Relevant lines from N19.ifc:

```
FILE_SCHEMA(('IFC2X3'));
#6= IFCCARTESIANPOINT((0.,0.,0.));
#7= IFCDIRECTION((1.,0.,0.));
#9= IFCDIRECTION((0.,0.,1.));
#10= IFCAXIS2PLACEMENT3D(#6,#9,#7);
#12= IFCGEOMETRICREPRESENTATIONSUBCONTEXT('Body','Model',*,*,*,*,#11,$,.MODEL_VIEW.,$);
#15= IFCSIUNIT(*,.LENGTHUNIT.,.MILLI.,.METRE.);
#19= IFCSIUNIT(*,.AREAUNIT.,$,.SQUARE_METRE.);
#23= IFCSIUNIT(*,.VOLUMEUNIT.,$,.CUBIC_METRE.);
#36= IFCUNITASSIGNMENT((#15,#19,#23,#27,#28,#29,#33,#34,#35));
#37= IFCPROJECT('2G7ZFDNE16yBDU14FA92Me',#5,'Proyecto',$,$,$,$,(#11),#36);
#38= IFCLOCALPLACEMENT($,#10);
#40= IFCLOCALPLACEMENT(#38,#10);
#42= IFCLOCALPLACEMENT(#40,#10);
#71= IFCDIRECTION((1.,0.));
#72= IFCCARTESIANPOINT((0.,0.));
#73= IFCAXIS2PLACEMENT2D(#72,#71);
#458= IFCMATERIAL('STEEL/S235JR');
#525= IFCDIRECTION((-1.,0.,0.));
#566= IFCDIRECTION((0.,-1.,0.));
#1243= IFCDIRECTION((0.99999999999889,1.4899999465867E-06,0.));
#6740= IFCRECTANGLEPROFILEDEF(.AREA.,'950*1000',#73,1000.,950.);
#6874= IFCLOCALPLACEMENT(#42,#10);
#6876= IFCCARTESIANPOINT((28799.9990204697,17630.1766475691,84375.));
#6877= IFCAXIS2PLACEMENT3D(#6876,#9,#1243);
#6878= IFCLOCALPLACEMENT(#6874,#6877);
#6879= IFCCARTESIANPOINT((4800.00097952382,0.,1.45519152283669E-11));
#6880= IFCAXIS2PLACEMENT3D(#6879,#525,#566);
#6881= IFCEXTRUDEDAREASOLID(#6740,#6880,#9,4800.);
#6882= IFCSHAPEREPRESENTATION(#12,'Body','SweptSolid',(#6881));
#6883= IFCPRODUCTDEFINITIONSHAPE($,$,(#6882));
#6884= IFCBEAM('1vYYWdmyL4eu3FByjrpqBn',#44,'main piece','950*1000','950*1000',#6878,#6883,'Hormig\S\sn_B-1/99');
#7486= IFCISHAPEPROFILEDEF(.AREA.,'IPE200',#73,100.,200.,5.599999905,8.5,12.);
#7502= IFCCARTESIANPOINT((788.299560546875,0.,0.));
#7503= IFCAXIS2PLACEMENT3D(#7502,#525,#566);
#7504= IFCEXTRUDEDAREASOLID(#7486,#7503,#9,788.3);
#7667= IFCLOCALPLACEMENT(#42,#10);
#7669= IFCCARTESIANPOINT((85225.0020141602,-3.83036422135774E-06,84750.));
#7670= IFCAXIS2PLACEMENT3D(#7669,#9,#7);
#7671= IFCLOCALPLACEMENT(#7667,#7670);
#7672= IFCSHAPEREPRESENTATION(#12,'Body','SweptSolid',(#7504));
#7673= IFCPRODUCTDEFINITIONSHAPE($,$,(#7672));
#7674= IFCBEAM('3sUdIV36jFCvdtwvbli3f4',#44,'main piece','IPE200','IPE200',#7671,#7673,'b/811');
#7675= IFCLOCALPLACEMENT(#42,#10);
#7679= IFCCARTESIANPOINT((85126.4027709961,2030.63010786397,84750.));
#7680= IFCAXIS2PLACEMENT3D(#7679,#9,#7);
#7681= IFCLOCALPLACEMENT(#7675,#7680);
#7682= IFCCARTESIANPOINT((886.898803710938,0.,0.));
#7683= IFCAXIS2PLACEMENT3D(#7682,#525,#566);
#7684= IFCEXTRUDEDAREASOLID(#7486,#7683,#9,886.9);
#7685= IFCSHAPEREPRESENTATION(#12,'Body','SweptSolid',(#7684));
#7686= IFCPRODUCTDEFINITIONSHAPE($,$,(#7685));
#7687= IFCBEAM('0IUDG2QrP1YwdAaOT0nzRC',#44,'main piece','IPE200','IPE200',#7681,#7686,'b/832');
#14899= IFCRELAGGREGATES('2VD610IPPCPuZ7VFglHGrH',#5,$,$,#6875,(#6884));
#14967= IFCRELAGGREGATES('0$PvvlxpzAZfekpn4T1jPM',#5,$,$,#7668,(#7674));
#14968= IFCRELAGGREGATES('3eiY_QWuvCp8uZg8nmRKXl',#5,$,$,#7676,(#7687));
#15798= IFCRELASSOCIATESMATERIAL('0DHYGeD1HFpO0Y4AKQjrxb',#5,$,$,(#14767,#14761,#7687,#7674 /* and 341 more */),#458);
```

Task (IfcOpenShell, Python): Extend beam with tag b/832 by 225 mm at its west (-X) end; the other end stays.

```python
import ifcopenshell
import ifcopenshell.util.representation
import ifcopenshell.util.unit

model = ifcopenshell.open("N19.ifc")
unit_scale = ifcopenshell.util.unit.calculate_unit_scale(model)

member = model.by_guid("0IUDG2QrP1YwdAaOT0nzRC")
change = 0.225 / unit_scale

# The extrusion runs towards the end named, so only its depth changes.
body = ifcopenshell.util.representation.get_representation(member, "Model", "Body")
solid = body.Items[0]
old_length = solid.Depth
solid.Depth += change

print(f"length {old_length:g} -> {solid.Depth:g}")

model.write("N19_edited.ifc")
```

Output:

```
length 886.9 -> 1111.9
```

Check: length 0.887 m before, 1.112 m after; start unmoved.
